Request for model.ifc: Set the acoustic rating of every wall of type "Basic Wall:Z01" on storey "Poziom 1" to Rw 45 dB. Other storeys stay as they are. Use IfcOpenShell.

First a look at what the model holds.

```python
import ifcopenshell
import ifcopenshell.util.element

model = ifcopenshell.open("model.ifc")
print(model.schema)
storey = next(s for s in model.by_type("IfcBuildingStorey") if s.Name == "Poziom 1")
walls = [e for e in ifcopenshell.util.element.get_decomposition(storey) if e.is_a("IfcWall")]
seen = {}
for e in walls:
    element_type = ifcopenshell.util.element.get_type(e)
    key = (element_type.Name if element_type != e and element_type else None, ifcopenshell.util.element.get_pset(e, "Pset_WallCommon", "AcousticRating"))
    seen[key] = seen.get(key, 0) + 1
for (name, value), count in sorted(seen.items(), key=str):
    print(count, "x", name, "|", value)
```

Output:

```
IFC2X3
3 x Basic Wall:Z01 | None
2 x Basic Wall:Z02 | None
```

```python
import ifcopenshell
import ifcopenshell.api.pset
import ifcopenshell.util.element

model = ifcopenshell.open("model.ifc")

storey = next(s for s in model.by_type("IfcBuildingStorey") if s.Name == "Poziom 1")
walls = [e for e in ifcopenshell.util.element.get_decomposition(storey) if e.is_a("IfcWall")]

count = 0
for e in walls:
    element_type = ifcopenshell.util.element.get_type(e)
    if element_type in (None, e) or element_type.Name != "Basic Wall:Z01":
        continue
    # add_pset returns the element's existing set when there is one.
    pset = ifcopenshell.api.pset.add_pset(model, product=e, name="Pset_WallCommon")
    ifcopenshell.api.pset.edit_pset(model, pset=pset, properties={"AcousticRating": "Rw 45 dB"})
    count += 1

print(count, "walls updated")

model.write("model_rev.ifc")
```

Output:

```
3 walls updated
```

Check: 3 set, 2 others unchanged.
